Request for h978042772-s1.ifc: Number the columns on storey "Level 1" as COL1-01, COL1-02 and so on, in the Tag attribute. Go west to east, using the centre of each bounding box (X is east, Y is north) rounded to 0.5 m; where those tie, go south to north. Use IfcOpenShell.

First a look at what the model holds.

```python
import ifcopenshell
import ifcopenshell.util.element
import ifcopenshell.util.placement

model = ifcopenshell.open("h978042772-s1.ifc")
print(model.schema)
storey = next(s for s in model.by_type("IfcBuildingStorey") if s.Name == "Level 1")
columns = [e for e in ifcopenshell.util.element.get_decomposition(storey) if e.is_a("IfcColumn")]
for e in sorted(columns, key=lambda e: e.id()):
    origin = ifcopenshell.util.placement.get_local_placement(e.ObjectPlacement)[:3, 3]
    print(e.id(), e.Tag, e.Name, origin.round(2) + 0.0, sep=" | ")
```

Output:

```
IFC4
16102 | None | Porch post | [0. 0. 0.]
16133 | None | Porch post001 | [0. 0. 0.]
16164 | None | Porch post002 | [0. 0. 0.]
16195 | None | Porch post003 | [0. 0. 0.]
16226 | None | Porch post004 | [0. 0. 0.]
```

```python
import ifcopenshell
import ifcopenshell.geom
import ifcopenshell.util.element
import ifcopenshell.util.shape

model = ifcopenshell.open("h978042772-s1.ifc")
settings = ifcopenshell.geom.settings()
settings.set("use-world-coords", True)


def centre(element):
    shape = ifcopenshell.geom.create_shape(settings, element)
    return ifcopenshell.util.shape.get_bbox_centroid(shape.geometry)


storey = next(s for s in model.by_type("IfcBuildingStorey") if s.Name == "Level 1")
columns = [e for e in ifcopenshell.util.element.get_decomposition(storey) if e.is_a("IfcColumn")]

# Insertion points can sit at a corner or the storey origin, so sort by the geometry (in metres).
centres = {e: centre(e) for e in columns}
columns.sort(key=lambda e: (round(centres[e][0] / 0.5), centres[e][1]))

for i, e in enumerate(columns, start=1):
    number = f"COL1-{i:02d}"
    e.Tag = number
    print(e.id(), number)

model.write("h978042772-s1-out.ifc")
```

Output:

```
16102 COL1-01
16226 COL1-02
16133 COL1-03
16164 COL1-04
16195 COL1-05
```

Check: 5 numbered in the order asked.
